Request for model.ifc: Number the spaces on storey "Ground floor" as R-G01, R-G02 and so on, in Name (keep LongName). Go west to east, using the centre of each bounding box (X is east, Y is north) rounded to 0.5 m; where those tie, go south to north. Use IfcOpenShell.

First a look at what the model holds.

```python
import ifcopenshell
import ifcopenshell.util.element
import ifcopenshell.util.placement

model = ifcopenshell.open("model.ifc")
print(model.schema)
storey = next(s for s in model.by_type("IfcBuildingStorey") if s.Name == "Ground floor")
spaces = [e for e in ifcopenshell.util.element.get_decomposition(storey) if e.is_a("IfcSpace")]
for e in sorted(spaces, key=lambda e: e.id()):
    origin = ifcopenshell.util.placement.get_local_placement(e.ObjectPlacement)[:3, 3]
    print(e.id(), e.Name, e.LongName, origin.round(2) + 0.0, sep=" | ")
```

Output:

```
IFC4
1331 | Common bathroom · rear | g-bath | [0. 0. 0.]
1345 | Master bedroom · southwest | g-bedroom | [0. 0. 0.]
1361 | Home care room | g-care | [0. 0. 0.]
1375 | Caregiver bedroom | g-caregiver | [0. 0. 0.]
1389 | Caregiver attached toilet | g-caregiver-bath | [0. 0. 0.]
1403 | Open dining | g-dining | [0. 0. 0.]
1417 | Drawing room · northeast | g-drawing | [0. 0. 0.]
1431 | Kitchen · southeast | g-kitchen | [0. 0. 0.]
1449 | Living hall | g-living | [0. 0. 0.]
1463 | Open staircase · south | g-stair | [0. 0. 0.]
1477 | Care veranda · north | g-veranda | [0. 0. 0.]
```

```python
import ifcopenshell
import ifcopenshell.geom
import ifcopenshell.util.element
import ifcopenshell.util.shape

model = ifcopenshell.open("model.ifc")
settings = ifcopenshell.geom.settings()
settings.set("use-world-coords", True)


def centre(element):
    shape = ifcopenshell.geom.create_shape(settings, element)
    return ifcopenshell.util.shape.get_bbox_centroid(shape.geometry)


storey = next(s for s in model.by_type("IfcBuildingStorey") if s.Name == "Ground floor")
spaces = [e for e in ifcopenshell.util.element.get_decomposition(storey) if e.is_a("IfcSpace")]

# Insertion points can sit at a corner or the storey origin, so sort by the geometry (in metres).
centres = {e: centre(e) for e in spaces}
spaces.sort(key=lambda e: (round(centres[e][0] / 0.5), centres[e][1]))

for i, e in enumerate(spaces, start=1):
    number = f"R-G{i:02d}"
    e.Name = number
    print(e.id(), number)

model.write("model_edited.ifc")
```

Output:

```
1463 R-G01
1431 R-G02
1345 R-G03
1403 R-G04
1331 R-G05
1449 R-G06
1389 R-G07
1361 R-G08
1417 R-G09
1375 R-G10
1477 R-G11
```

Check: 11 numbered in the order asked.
